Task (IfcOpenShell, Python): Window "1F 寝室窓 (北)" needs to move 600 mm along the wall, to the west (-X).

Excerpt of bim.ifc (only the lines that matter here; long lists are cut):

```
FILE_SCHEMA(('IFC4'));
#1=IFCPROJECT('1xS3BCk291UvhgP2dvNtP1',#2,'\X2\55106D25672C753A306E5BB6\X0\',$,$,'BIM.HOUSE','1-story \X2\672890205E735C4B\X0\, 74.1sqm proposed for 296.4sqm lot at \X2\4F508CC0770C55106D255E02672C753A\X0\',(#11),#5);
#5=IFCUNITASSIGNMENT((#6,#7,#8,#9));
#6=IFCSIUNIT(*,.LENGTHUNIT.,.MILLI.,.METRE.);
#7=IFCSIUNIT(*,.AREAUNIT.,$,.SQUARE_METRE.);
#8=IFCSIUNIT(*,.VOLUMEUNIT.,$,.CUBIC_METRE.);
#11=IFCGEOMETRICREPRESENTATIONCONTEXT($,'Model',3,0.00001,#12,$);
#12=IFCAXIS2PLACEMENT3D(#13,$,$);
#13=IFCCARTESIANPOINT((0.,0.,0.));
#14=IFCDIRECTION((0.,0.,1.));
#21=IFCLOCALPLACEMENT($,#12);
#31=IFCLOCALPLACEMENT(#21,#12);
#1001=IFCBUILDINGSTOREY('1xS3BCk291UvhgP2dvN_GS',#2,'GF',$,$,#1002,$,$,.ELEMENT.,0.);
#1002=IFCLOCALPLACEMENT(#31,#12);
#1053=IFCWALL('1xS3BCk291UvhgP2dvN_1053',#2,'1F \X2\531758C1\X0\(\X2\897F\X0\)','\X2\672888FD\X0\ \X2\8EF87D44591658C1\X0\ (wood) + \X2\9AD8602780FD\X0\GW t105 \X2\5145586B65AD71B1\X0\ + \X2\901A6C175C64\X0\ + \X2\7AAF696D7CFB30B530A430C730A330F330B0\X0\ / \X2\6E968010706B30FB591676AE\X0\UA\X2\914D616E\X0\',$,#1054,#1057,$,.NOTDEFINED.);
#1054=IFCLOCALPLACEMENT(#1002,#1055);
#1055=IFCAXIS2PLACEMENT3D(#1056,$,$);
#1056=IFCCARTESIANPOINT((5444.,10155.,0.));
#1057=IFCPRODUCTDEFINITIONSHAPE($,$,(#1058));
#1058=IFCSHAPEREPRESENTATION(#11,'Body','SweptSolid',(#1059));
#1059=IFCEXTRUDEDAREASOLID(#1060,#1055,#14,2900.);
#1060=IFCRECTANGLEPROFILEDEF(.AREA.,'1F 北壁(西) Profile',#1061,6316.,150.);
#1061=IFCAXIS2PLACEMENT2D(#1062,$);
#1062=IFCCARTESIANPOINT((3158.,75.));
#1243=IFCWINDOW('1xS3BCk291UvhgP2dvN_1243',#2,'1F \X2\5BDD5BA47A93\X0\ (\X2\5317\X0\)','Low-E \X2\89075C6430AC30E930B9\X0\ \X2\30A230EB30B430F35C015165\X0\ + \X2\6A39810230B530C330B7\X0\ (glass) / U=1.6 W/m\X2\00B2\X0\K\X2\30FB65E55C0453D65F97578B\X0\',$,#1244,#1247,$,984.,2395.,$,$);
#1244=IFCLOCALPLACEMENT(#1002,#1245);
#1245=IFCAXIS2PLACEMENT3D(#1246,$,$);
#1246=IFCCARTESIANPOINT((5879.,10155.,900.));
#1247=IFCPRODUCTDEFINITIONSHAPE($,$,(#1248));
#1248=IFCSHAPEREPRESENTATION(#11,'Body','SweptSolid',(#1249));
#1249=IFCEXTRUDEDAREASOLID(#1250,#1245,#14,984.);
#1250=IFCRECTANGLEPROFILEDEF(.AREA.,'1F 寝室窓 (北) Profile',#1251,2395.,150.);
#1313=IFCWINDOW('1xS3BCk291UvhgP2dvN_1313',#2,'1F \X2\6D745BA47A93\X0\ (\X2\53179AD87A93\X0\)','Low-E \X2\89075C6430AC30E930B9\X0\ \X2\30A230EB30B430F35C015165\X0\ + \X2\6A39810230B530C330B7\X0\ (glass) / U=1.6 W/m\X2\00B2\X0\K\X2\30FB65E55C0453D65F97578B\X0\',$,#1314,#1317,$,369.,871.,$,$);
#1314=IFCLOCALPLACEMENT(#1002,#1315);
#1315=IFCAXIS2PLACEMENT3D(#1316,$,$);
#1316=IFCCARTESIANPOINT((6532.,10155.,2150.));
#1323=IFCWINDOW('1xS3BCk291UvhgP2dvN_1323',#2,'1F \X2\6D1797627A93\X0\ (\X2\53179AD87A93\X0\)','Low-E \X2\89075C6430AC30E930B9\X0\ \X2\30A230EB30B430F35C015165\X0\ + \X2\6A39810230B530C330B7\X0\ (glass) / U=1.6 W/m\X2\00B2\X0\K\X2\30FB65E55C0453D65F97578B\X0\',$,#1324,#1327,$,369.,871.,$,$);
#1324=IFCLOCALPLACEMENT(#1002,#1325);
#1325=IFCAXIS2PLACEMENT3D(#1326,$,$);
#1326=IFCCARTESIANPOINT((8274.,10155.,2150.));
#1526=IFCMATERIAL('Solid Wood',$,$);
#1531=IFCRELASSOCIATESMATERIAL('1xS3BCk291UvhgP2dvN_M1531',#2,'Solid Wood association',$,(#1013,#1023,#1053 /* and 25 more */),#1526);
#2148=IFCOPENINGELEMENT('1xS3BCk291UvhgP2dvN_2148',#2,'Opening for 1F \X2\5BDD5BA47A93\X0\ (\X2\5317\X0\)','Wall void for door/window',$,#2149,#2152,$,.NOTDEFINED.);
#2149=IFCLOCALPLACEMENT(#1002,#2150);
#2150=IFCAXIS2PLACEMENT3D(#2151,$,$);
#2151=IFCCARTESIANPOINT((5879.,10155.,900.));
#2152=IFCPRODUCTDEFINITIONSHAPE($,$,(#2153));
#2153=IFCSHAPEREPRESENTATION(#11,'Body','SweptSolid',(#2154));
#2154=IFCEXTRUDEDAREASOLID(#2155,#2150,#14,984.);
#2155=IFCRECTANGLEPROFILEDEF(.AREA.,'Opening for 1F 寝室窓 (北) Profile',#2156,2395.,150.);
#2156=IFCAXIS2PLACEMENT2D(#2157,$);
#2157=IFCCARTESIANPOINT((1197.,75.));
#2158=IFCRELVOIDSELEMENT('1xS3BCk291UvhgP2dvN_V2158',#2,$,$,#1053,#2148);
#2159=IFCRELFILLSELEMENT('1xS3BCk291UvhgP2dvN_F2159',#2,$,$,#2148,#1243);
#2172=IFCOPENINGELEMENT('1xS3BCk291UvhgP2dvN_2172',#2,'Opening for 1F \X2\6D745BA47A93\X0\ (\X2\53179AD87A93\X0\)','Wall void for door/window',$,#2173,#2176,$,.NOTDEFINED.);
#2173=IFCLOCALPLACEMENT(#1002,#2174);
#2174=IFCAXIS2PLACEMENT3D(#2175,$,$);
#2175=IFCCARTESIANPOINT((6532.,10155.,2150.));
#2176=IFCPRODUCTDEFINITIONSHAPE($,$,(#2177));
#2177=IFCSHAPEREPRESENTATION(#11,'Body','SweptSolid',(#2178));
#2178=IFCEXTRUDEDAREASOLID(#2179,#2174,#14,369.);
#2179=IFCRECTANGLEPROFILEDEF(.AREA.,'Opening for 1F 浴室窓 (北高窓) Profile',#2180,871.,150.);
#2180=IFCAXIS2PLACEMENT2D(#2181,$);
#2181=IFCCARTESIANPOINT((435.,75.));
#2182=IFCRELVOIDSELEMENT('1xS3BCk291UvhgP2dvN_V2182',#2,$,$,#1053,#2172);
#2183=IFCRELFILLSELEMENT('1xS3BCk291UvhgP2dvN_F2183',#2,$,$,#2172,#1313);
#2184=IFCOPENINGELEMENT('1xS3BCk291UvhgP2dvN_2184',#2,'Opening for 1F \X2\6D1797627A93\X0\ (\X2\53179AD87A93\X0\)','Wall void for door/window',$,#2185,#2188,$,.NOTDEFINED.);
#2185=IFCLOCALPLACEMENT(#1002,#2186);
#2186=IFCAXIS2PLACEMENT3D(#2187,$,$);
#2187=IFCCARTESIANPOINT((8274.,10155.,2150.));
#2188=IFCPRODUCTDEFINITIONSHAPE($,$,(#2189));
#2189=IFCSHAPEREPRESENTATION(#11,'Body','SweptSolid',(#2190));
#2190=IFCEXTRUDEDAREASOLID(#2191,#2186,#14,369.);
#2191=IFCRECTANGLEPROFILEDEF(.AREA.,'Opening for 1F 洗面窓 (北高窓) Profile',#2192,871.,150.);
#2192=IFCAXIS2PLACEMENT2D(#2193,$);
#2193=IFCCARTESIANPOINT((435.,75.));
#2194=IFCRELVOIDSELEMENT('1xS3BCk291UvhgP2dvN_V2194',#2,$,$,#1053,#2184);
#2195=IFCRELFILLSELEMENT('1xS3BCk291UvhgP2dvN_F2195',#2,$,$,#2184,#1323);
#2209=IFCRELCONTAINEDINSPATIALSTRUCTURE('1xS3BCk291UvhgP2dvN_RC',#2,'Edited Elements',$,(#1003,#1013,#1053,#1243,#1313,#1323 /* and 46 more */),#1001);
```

```python
import ifcopenshell
import ifcopenshell.api.geometry
import ifcopenshell.util.placement
import ifcopenshell.util.unit

model = ifcopenshell.open("bim.ifc")
unit_scale = ifcopenshell.util.unit.calculate_unit_scale(model)

window = model.by_guid("1xS3BCk291UvhgP2dvN_1243")
opening = window.FillsVoids[0].RelatingOpeningElement
wall = opening.VoidsElements[0].RelatingBuildingElement

wall_matrix = ifcopenshell.util.placement.get_local_placement(wall.ObjectPlacement)
shift = wall_matrix[:3, 0] * -0.6 / unit_scale
before = ifcopenshell.util.placement.get_local_placement(window.ObjectPlacement)[:3, 3].copy()

# The window is not placed relative to its opening, so move both.
for product in (opening, window):
    matrix = ifcopenshell.util.placement.get_local_placement(product.ObjectPlacement)
    matrix[:3, 3] += shift
    ifcopenshell.api.geometry.edit_object_placement(model, product=product, matrix=matrix, is_si=False)

after = ifcopenshell.util.placement.get_local_placement(window.ObjectPlacement)[:3, 3]
print("window moved by", (after - before).round(3) + 0.0)

model.write("bim_v2.ifc")
```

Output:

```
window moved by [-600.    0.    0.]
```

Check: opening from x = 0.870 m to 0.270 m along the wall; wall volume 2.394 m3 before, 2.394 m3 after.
